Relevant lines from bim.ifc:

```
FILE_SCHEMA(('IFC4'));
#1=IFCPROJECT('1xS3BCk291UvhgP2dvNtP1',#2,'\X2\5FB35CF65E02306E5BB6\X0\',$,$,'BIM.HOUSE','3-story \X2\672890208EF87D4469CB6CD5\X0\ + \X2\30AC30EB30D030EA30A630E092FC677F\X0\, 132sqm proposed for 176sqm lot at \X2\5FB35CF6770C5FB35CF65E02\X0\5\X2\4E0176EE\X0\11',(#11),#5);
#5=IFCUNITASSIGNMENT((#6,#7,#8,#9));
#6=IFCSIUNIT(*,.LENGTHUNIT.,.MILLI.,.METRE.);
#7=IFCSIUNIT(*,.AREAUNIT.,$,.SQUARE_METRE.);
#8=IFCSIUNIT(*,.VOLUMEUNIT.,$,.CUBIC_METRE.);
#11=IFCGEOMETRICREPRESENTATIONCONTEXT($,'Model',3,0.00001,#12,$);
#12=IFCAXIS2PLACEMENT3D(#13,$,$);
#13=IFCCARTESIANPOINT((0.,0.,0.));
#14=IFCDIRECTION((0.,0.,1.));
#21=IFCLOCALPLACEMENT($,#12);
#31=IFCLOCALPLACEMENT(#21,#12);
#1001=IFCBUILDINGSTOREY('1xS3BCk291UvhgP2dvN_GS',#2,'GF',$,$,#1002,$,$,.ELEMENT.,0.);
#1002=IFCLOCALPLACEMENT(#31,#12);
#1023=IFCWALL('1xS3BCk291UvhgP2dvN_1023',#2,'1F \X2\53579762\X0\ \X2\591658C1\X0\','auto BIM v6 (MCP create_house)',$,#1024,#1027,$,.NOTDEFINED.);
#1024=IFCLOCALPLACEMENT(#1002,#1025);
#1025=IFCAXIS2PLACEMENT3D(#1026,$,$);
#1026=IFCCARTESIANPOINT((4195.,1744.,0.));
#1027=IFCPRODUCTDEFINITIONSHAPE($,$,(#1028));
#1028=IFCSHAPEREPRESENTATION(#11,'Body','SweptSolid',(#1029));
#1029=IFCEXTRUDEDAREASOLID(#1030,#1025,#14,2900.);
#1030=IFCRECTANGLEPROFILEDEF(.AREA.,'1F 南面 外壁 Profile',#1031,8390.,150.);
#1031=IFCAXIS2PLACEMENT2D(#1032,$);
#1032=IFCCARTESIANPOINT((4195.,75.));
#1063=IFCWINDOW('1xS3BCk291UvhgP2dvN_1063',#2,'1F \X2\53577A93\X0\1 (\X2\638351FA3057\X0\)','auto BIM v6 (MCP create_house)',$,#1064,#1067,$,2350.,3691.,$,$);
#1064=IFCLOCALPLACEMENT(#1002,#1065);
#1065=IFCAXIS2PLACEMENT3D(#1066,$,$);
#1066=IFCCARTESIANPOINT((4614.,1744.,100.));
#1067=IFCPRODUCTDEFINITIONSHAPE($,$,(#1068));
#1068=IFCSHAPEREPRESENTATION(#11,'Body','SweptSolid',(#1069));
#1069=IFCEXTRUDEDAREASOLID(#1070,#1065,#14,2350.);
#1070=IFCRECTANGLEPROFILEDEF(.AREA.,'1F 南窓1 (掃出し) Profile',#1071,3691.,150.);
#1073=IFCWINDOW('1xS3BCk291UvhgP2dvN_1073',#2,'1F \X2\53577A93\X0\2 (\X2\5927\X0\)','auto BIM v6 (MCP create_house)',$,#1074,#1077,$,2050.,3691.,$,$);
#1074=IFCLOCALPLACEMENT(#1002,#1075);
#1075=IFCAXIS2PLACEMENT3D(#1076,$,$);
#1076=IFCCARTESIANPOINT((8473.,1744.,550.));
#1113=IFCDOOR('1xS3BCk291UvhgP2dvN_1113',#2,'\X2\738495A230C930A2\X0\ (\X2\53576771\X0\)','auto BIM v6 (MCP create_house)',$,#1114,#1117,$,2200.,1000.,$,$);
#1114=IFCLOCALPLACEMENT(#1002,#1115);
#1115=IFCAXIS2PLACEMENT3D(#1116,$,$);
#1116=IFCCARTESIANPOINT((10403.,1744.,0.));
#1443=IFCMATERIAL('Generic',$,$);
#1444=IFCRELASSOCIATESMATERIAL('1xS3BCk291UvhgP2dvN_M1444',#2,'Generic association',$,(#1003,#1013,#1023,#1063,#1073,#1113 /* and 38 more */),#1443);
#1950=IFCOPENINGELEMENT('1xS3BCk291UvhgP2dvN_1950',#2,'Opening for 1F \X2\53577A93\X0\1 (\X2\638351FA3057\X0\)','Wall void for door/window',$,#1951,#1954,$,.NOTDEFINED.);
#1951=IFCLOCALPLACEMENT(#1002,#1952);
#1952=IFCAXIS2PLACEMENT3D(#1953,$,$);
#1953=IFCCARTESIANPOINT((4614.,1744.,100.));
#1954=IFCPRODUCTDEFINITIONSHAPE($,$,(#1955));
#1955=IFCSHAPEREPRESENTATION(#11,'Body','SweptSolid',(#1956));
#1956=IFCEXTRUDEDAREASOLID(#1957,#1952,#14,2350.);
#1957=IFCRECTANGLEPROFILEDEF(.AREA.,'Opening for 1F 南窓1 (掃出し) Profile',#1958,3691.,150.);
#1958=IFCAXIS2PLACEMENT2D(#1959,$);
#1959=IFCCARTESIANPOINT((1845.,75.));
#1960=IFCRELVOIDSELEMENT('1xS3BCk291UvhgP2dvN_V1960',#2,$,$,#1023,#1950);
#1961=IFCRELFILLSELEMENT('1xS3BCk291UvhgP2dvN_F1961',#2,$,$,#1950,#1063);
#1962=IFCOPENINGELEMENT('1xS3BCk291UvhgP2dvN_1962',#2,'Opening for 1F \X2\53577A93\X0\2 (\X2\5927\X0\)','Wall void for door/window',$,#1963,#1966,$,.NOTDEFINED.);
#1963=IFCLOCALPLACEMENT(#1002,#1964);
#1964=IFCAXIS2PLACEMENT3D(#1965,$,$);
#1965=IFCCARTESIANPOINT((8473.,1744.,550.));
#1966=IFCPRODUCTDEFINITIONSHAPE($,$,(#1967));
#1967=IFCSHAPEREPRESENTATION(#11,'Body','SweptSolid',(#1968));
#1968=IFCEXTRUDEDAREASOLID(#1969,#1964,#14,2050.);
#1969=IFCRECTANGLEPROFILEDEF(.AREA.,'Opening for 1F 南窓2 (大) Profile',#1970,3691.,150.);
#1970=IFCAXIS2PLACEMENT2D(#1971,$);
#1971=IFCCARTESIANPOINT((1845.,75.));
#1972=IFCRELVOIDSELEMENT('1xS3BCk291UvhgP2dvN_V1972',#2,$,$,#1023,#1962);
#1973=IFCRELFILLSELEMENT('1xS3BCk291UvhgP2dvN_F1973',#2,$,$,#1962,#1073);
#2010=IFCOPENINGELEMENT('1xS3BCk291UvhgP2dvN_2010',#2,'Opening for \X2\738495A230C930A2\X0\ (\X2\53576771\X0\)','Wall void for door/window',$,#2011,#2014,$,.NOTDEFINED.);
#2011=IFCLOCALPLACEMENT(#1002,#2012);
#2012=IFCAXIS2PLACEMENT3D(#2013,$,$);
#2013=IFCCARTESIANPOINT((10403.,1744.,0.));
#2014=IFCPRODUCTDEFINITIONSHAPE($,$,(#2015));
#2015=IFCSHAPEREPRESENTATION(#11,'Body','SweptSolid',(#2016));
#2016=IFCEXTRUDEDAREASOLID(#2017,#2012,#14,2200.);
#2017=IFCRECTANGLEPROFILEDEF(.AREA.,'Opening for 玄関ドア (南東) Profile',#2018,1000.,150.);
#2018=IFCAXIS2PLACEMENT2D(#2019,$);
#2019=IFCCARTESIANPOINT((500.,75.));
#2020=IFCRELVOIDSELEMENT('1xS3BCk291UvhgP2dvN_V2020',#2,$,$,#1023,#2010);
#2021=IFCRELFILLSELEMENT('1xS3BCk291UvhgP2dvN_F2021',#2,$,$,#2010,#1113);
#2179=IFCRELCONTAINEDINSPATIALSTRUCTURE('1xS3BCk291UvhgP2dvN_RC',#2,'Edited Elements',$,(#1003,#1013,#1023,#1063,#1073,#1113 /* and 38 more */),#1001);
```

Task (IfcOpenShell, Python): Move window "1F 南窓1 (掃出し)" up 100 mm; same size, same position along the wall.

```python
import numpy as np
import ifcopenshell
import ifcopenshell.api.geometry
import ifcopenshell.util.placement
import ifcopenshell.util.unit

model = ifcopenshell.open("bim.ifc")
unit_scale = ifcopenshell.util.unit.calculate_unit_scale(model)

window = model.by_guid("1xS3BCk291UvhgP2dvN_1063")
opening = window.FillsVoids[0].RelatingOpeningElement
dz = 100.0

shift = np.array([0.0, 0.0, dz])
# The window is not placed relative to its opening, so move both.
for product in (opening, window):
    matrix = ifcopenshell.util.placement.get_local_placement(product.ObjectPlacement)
    matrix[:3, 3] += shift
    ifcopenshell.api.geometry.edit_object_placement(model, product=product, matrix=matrix, is_si=False)

print(f"moved by {dz * unit_scale:+.3f} m")

model.write("bim_v2.ifc")
```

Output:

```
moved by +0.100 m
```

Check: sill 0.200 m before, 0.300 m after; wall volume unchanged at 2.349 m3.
